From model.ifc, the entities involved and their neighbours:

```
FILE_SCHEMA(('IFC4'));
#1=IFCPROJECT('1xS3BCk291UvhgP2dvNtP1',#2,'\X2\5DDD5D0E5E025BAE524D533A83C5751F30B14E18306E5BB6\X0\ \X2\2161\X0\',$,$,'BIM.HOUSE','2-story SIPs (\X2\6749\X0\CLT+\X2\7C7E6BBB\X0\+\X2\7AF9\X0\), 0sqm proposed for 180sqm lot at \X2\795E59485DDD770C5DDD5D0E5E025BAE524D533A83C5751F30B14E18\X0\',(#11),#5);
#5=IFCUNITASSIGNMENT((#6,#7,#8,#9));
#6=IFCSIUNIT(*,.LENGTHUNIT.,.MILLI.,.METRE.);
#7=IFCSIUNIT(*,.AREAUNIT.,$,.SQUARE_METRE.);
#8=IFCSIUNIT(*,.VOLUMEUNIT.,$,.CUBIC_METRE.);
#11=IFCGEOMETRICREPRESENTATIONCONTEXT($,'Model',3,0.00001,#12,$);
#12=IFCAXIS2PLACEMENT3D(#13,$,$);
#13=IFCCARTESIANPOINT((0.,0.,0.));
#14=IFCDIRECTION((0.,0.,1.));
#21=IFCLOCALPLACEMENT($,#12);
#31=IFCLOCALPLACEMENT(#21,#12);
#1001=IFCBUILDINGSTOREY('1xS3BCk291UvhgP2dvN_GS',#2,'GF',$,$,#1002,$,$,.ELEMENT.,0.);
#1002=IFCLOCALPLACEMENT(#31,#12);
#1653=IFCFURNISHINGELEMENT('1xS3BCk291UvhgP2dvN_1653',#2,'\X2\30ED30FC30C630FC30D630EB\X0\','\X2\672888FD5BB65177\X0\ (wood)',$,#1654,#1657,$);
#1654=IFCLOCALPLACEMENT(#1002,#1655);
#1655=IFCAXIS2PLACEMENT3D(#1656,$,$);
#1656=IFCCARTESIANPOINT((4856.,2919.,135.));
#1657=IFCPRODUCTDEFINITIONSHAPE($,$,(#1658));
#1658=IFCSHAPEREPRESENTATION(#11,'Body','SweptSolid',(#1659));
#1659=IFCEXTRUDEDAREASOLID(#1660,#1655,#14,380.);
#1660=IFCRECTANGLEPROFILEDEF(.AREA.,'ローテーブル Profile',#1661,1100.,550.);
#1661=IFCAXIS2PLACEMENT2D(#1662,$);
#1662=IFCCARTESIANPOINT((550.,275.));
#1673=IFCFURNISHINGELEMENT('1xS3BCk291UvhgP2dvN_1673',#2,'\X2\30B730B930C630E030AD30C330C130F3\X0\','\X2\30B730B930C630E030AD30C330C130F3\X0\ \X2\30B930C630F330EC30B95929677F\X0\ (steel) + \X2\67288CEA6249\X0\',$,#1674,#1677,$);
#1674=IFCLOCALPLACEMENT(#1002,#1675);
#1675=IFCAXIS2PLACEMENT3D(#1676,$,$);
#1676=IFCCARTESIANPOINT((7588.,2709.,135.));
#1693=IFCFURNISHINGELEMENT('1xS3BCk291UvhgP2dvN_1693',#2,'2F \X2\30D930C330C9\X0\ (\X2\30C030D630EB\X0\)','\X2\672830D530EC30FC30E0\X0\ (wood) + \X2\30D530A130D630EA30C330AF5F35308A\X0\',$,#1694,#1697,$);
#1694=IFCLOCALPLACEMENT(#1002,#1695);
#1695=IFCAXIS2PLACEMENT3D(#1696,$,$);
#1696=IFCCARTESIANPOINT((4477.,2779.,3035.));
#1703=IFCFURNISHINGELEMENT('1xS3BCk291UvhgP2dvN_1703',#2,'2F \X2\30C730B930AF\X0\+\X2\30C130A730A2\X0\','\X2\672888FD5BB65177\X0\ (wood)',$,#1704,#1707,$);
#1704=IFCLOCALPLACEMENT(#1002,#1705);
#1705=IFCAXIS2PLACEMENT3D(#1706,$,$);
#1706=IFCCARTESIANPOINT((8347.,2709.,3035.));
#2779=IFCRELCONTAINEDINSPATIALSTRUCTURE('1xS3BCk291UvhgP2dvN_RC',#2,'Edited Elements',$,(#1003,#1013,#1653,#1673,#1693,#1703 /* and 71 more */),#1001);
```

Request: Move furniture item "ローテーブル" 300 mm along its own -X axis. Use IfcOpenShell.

```python
import ifcopenshell
import ifcopenshell.api.geometry
import ifcopenshell.util.placement

model = ifcopenshell.open("model.ifc")

item = model.by_guid("1xS3BCk291UvhgP2dvN_1653")
matrix = ifcopenshell.util.placement.get_local_placement(item.ObjectPlacement)
matrix[:3, 3] -= matrix[:3, 0] * 300.0
ifcopenshell.api.geometry.edit_object_placement(model, product=item, matrix=matrix, is_si=False)

print(ifcopenshell.util.placement.get_local_placement(item.ObjectPlacement).round(3) + 0.0)

model.write("model_rev.ifc")
```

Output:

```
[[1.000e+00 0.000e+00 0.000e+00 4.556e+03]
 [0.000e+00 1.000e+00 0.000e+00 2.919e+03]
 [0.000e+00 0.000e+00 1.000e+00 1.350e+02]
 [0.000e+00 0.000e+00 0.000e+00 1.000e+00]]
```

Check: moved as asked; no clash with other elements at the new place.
